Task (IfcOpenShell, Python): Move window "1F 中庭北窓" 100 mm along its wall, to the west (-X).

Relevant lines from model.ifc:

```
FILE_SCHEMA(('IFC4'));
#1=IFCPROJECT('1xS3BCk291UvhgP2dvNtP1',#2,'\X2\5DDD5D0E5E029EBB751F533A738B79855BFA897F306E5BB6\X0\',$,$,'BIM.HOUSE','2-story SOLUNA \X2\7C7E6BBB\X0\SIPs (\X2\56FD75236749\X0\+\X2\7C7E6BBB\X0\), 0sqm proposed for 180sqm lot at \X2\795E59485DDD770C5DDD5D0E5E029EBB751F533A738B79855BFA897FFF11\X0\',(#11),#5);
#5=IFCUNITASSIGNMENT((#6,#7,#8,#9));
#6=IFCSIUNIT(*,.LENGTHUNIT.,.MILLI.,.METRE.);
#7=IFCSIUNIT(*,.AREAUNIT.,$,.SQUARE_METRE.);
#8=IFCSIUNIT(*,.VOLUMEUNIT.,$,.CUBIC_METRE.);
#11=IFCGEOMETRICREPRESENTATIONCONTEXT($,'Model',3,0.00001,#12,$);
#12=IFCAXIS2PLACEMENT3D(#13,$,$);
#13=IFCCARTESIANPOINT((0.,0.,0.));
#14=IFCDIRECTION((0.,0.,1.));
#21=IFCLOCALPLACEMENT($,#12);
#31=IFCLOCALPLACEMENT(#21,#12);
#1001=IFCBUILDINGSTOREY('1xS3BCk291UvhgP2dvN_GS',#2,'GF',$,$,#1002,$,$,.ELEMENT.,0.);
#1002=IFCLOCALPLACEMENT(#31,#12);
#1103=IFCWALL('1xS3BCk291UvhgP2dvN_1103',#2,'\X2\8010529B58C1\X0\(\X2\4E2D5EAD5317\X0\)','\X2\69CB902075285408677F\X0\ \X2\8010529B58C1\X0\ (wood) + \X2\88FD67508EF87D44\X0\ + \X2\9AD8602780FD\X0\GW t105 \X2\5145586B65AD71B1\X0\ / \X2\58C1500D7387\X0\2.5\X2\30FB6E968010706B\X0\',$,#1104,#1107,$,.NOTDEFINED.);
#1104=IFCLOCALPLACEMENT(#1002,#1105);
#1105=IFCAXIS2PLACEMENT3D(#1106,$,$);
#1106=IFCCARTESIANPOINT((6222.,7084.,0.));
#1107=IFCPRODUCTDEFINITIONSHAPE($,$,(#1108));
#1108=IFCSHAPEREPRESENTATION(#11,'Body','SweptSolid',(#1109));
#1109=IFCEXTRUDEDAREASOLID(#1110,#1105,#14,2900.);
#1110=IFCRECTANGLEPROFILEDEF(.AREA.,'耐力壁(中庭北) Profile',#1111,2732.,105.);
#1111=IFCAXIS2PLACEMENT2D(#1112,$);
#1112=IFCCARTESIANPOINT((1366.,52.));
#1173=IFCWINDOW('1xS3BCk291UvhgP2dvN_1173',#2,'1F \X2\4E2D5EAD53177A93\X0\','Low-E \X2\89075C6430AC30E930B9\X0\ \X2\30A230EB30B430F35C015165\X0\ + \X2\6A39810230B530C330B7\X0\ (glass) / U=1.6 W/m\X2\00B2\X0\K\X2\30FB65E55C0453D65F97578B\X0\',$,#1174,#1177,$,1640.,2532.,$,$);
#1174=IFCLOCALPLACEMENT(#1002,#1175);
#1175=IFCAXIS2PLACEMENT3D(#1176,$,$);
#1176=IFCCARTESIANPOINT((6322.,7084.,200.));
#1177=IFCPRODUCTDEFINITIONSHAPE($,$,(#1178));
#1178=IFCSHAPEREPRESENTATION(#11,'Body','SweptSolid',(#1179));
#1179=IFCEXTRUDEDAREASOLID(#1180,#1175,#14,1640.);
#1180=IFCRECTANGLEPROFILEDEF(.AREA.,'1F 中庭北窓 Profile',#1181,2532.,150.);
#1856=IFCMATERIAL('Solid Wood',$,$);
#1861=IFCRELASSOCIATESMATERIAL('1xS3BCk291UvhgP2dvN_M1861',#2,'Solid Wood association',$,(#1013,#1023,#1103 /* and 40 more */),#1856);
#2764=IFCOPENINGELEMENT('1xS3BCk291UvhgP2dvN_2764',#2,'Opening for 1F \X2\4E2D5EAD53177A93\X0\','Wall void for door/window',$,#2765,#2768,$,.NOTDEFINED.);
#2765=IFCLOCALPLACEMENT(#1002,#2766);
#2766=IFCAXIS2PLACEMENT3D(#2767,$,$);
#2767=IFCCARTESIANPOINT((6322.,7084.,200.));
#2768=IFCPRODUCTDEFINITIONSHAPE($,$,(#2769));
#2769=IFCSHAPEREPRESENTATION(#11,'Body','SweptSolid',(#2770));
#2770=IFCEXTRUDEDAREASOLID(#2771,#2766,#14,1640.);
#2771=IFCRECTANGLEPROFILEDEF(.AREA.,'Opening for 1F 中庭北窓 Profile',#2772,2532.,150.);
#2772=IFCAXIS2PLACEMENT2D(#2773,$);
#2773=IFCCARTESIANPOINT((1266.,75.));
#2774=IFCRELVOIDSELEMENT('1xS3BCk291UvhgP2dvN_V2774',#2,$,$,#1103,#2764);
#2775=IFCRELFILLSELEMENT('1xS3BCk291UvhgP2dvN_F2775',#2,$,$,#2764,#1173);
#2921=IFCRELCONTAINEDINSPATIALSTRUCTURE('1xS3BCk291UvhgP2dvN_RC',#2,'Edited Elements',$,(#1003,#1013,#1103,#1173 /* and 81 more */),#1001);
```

```python
import ifcopenshell
import ifcopenshell.api.geometry
import ifcopenshell.util.placement

model = ifcopenshell.open("model.ifc")

window = model.by_guid("1xS3BCk291UvhgP2dvN_1173")
opening = window.FillsVoids[0].RelatingOpeningElement
wall = opening.VoidsElements[0].RelatingBuildingElement

wall_matrix = ifcopenshell.util.placement.get_local_placement(wall.ObjectPlacement)
shift = wall_matrix[:3, 0] * -100.0
before = ifcopenshell.util.placement.get_local_placement(window.ObjectPlacement)[:3, 3].copy()

# The window is not placed relative to its opening, so move both.
for product in (opening, window):
    matrix = ifcopenshell.util.placement.get_local_placement(product.ObjectPlacement)
    matrix[:3, 3] += shift
    ifcopenshell.api.geometry.edit_object_placement(model, product=product, matrix=matrix, is_si=False)

after = ifcopenshell.util.placement.get_local_placement(window.ObjectPlacement)[:3, 3]
print("window moved by", (after - before).round(3) + 0.0)

model.write("model-out.ifc")
```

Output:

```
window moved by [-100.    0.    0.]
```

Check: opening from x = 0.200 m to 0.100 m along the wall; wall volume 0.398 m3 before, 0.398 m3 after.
